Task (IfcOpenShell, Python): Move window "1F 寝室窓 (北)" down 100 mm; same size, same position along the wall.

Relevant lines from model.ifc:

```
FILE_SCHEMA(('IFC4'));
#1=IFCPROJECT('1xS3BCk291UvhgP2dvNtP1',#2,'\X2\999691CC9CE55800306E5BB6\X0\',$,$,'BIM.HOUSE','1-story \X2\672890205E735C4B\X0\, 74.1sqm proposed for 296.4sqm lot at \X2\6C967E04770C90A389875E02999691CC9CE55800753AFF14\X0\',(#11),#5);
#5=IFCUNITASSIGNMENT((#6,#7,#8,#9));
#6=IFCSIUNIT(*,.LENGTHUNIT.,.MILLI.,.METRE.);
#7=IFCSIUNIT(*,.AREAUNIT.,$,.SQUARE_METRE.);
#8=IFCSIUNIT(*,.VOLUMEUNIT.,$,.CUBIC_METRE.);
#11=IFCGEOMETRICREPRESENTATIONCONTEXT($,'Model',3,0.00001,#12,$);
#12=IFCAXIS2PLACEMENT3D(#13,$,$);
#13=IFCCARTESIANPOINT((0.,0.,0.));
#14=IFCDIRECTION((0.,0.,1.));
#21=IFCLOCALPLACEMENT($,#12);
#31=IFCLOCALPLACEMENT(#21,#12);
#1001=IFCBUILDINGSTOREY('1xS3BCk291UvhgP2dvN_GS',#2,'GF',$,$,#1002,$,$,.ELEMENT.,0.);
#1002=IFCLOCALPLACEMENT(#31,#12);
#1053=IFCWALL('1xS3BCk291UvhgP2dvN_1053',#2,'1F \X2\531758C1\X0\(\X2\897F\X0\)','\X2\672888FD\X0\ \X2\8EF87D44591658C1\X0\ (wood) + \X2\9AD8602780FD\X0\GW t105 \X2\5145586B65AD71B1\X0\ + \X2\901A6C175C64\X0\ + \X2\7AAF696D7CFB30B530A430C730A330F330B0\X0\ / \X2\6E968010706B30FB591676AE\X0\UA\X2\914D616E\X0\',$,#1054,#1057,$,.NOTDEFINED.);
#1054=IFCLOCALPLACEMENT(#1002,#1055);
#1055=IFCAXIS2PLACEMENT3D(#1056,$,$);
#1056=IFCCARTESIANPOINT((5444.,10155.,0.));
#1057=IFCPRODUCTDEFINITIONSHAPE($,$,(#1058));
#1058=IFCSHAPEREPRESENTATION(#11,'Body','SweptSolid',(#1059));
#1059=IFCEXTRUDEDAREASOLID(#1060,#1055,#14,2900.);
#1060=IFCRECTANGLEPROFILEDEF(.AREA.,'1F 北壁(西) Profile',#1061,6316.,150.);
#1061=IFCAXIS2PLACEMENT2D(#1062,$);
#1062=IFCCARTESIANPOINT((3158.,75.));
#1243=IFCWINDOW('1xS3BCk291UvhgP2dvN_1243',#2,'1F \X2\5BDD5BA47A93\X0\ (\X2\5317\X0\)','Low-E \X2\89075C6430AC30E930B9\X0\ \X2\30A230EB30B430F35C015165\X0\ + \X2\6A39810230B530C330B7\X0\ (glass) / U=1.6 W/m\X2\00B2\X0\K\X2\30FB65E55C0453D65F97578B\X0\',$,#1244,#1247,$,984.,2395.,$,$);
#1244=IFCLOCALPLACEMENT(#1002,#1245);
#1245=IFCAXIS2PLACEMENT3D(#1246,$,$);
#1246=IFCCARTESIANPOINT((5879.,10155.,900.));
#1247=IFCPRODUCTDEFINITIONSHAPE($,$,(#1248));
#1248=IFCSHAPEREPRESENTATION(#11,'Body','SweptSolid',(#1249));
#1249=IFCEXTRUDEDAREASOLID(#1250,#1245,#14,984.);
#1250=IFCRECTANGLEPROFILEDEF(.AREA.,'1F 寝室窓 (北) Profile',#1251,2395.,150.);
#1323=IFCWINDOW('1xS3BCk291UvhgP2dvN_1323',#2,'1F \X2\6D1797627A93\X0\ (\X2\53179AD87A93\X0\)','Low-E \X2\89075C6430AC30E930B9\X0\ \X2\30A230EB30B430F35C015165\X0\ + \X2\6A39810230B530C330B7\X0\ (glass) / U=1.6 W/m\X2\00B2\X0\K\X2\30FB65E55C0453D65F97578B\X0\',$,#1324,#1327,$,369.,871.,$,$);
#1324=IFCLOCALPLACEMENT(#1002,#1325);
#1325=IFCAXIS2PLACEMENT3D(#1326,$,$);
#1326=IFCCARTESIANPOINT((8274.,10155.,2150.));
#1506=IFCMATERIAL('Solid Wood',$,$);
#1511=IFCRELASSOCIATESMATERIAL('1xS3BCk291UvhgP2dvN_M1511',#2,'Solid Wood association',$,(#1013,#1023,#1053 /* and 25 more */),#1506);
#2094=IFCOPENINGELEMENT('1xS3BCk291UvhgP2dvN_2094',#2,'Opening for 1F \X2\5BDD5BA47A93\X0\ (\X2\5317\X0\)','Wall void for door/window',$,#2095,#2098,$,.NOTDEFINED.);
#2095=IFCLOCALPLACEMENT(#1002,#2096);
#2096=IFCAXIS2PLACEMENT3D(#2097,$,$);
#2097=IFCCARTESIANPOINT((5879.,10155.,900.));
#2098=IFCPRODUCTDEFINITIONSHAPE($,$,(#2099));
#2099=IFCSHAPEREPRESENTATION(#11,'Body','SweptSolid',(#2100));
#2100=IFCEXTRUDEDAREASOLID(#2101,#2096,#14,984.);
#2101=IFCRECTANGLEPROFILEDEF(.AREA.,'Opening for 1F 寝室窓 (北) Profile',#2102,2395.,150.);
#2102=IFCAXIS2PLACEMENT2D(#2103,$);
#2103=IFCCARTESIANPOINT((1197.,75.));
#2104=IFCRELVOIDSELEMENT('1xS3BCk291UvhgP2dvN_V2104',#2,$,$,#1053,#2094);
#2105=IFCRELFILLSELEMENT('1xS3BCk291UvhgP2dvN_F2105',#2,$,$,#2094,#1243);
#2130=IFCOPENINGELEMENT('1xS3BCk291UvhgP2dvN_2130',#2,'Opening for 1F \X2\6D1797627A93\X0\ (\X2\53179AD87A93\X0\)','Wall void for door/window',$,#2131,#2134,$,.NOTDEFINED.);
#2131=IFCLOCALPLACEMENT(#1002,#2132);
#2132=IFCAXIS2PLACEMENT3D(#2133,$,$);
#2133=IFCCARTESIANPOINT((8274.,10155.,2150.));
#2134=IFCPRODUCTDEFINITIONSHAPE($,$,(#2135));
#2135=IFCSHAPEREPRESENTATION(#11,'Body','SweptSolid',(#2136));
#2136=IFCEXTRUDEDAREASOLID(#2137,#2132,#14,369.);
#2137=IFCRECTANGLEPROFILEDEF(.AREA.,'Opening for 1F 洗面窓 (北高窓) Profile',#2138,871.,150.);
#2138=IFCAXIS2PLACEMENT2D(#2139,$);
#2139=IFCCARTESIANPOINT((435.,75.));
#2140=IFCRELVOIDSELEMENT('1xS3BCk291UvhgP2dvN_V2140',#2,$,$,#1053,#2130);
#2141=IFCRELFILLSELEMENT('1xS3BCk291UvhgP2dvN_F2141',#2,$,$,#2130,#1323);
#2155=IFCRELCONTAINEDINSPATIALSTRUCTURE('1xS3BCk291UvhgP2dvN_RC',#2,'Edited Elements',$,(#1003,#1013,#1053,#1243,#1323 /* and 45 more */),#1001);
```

```python
import numpy as np
import ifcopenshell
import ifcopenshell.api.geometry
import ifcopenshell.util.placement
import ifcopenshell.util.unit

model = ifcopenshell.open("model.ifc")
unit_scale = ifcopenshell.util.unit.calculate_unit_scale(model)

window = model.by_guid("1xS3BCk291UvhgP2dvN_1243")
opening = window.FillsVoids[0].RelatingOpeningElement
dz = -100.0

shift = np.array([0.0, 0.0, dz])
# The window is not placed relative to its opening, so move both.
for product in (opening, window):
    matrix = ifcopenshell.util.placement.get_local_placement(product.ObjectPlacement)
    matrix[:3, 3] += shift
    ifcopenshell.api.geometry.edit_object_placement(model, product=product, matrix=matrix, is_si=False)

print(f"moved by {dz * unit_scale:+.3f} m")

model.write("model_edited.ifc")
```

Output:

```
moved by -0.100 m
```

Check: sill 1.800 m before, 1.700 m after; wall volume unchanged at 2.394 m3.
